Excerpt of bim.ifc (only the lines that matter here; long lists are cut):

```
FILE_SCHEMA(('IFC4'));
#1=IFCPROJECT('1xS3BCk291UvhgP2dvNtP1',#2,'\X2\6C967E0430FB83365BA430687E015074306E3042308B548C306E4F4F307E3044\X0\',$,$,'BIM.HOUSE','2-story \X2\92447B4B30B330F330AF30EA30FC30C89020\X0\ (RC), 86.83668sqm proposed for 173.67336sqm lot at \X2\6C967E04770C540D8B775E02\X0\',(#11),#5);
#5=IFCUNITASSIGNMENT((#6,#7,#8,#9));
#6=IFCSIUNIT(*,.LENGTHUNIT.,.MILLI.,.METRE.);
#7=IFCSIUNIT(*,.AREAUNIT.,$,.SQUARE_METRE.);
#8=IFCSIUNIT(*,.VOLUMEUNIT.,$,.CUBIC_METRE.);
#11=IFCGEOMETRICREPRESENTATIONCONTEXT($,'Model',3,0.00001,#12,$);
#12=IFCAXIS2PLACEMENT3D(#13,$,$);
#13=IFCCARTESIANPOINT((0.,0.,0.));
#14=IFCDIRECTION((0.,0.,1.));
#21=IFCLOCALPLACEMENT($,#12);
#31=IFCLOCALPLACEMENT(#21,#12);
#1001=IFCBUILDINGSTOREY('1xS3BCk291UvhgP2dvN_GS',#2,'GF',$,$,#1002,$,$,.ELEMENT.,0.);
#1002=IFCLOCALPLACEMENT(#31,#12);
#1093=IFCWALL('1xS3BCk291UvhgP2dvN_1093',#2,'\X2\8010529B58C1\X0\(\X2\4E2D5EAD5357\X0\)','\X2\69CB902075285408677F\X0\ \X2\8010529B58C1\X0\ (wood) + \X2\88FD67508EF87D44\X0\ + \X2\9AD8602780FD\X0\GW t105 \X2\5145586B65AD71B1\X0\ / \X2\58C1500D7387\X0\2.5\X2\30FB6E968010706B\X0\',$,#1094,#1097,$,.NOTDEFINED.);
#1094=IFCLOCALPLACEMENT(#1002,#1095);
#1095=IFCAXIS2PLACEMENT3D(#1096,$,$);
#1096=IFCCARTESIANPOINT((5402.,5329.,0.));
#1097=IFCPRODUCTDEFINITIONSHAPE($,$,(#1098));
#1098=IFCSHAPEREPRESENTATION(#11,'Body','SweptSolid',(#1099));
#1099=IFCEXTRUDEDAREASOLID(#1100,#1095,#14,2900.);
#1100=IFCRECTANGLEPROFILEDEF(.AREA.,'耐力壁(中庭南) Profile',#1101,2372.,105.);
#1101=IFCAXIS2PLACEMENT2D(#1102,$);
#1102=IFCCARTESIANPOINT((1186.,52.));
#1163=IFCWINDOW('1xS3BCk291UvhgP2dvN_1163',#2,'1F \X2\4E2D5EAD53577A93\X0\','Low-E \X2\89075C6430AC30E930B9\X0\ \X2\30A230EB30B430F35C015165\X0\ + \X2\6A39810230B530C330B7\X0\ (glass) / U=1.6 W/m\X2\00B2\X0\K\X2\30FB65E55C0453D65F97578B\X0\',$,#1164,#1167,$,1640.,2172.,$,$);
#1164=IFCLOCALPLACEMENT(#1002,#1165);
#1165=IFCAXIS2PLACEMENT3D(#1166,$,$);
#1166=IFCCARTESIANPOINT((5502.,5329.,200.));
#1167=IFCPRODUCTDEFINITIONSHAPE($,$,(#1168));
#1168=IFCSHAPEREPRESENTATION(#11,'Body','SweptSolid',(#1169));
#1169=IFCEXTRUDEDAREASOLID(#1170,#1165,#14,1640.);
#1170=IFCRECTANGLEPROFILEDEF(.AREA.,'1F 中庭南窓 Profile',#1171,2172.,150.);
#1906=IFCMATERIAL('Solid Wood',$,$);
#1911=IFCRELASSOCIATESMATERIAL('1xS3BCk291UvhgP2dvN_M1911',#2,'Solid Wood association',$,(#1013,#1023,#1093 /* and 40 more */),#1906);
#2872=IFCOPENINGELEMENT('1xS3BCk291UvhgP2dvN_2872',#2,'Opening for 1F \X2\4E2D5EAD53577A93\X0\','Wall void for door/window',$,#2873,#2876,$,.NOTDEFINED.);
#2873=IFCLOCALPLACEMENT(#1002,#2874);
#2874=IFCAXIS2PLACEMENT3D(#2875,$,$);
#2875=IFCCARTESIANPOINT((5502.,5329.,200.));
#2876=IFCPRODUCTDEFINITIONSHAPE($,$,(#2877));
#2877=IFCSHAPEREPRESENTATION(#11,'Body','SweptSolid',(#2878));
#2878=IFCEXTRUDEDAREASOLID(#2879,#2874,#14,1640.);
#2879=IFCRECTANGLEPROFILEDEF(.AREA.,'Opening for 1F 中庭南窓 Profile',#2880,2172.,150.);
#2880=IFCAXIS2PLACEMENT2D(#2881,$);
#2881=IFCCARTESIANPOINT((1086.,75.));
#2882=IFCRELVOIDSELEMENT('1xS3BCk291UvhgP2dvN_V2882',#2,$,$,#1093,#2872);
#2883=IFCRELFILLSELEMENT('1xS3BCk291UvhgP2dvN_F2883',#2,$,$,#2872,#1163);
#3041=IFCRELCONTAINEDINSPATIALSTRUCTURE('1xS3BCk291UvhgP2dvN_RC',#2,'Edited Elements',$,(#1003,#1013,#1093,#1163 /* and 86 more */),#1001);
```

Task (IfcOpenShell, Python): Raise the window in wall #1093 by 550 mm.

```python
import numpy as np
import ifcopenshell
import ifcopenshell.api.geometry
import ifcopenshell.util.placement
import ifcopenshell.util.unit

model = ifcopenshell.open("bim.ifc")
unit_scale = ifcopenshell.util.unit.calculate_unit_scale(model)

window = model.by_id(1163)
opening = window.FillsVoids[0].RelatingOpeningElement
dz = 0.55 / unit_scale

shift = np.array([0.0, 0.0, dz])
# The window is not placed relative to its opening, so move both.
for product in (opening, window):
    matrix = ifcopenshell.util.placement.get_local_placement(product.ObjectPlacement)
    matrix[:3, 3] += shift
    ifcopenshell.api.geometry.edit_object_placement(model, product=product, matrix=matrix, is_si=False)

print(f"moved by {dz * unit_scale:+.3f} m")

model.write("bim_edited.ifc")
```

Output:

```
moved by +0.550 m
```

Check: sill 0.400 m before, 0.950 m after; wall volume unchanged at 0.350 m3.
